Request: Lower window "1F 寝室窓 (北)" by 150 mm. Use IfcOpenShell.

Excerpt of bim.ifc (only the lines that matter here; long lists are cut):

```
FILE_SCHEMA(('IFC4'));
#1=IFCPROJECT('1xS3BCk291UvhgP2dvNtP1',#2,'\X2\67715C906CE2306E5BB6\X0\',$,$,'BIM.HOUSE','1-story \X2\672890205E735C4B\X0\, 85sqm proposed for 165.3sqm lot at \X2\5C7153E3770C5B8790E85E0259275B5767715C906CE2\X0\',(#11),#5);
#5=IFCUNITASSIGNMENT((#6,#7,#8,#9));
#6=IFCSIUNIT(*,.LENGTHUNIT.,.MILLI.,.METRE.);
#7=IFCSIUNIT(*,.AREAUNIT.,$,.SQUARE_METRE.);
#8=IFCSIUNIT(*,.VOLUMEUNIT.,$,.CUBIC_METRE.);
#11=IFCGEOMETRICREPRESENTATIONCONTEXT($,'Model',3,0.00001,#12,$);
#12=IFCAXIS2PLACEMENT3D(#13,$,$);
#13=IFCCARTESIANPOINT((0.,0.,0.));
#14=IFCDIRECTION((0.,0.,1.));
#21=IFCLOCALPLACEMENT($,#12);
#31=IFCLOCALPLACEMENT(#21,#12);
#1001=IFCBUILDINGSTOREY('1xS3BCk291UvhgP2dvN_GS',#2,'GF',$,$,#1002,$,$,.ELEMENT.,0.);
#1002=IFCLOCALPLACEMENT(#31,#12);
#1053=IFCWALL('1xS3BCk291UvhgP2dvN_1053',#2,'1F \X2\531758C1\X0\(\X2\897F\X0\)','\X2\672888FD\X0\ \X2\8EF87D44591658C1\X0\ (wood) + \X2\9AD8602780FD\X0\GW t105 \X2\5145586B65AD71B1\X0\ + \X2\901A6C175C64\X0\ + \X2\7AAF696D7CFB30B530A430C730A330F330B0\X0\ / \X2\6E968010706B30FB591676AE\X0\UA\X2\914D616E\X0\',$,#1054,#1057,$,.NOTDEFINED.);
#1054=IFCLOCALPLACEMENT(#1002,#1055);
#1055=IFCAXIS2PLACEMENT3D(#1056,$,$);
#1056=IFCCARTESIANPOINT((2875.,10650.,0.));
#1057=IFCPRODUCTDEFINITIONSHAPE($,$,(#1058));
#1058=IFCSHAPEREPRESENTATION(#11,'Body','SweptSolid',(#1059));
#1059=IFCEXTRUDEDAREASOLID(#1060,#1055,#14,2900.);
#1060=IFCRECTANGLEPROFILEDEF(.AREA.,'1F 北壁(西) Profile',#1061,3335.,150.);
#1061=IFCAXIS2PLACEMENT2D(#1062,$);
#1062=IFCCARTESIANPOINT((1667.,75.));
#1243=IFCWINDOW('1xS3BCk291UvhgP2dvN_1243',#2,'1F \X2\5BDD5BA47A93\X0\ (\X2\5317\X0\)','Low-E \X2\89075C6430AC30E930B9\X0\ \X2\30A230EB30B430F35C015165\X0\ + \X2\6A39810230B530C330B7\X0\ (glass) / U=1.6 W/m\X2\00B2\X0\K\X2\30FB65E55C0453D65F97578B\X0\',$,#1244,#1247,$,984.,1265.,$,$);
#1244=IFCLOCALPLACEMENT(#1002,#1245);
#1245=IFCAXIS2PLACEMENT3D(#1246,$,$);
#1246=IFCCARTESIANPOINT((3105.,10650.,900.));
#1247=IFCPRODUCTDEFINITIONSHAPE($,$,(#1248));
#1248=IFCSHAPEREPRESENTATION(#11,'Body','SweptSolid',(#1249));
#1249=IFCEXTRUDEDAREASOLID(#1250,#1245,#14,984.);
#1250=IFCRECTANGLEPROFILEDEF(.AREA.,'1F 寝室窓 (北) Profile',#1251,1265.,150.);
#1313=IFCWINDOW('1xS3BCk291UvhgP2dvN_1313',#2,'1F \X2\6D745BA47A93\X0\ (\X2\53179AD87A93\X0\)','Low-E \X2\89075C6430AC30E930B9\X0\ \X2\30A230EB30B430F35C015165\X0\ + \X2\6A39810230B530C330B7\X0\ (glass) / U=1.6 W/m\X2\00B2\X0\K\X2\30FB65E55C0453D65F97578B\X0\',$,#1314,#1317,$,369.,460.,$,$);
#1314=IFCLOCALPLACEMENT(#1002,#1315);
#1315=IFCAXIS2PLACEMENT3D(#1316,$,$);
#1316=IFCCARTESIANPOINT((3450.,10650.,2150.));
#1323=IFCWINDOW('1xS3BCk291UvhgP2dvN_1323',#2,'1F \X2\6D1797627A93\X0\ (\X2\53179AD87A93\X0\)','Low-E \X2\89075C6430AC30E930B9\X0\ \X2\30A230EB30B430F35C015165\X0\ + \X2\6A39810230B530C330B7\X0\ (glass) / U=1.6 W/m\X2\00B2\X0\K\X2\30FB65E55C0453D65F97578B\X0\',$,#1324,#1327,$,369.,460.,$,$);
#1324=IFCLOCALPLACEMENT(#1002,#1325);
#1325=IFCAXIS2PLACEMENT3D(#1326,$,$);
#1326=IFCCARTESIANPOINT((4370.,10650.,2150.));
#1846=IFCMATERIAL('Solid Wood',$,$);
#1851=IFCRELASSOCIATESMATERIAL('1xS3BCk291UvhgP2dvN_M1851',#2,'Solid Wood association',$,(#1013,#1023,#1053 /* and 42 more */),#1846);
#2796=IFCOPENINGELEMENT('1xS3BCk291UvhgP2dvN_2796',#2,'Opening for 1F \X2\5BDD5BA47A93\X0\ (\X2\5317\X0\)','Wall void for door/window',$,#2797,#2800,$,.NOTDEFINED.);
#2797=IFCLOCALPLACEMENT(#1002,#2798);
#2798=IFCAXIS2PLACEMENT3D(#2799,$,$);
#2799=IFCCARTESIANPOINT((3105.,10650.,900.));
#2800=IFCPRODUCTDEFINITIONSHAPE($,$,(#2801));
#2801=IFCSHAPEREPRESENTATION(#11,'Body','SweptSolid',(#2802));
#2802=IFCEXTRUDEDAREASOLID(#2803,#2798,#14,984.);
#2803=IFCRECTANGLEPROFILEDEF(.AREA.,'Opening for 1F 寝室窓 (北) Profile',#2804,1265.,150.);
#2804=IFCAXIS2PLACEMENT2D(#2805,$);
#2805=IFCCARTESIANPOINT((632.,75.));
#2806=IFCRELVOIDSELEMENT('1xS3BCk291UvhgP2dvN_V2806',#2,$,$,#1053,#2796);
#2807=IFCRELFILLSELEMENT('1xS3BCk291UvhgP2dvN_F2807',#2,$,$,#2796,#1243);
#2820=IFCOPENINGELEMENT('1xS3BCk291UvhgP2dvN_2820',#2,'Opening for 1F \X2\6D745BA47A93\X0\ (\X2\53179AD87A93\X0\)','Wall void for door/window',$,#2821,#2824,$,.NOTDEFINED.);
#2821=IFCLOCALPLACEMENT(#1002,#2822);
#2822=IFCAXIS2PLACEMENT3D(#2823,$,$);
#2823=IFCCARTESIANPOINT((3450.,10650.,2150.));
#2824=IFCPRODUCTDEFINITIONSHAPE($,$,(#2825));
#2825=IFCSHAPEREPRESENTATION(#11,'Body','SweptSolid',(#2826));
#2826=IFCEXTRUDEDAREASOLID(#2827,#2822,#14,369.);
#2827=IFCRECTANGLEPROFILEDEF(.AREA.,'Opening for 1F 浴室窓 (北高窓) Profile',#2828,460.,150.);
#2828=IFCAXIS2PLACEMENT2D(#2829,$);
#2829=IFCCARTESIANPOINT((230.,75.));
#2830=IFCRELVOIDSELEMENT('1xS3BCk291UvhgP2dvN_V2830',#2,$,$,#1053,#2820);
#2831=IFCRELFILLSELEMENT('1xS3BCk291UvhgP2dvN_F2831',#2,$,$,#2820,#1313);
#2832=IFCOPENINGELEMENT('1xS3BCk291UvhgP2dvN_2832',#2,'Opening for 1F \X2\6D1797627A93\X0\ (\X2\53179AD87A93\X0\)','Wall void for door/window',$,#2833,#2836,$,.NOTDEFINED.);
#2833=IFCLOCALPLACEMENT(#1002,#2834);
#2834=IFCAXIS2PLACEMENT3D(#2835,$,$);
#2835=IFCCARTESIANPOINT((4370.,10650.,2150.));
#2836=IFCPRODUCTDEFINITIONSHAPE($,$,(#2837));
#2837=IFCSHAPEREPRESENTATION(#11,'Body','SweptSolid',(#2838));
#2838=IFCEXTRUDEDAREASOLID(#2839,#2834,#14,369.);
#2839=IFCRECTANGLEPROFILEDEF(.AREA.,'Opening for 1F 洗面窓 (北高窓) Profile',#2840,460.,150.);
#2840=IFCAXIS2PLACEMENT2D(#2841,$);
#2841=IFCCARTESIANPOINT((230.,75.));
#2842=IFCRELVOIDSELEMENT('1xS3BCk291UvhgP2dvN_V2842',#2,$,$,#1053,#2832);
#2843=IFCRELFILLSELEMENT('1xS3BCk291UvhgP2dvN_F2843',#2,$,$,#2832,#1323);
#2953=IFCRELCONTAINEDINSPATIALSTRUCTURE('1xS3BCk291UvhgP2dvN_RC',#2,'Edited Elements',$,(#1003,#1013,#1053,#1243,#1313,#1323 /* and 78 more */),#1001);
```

```python
import numpy as np
import ifcopenshell
import ifcopenshell.api.geometry
import ifcopenshell.util.placement
import ifcopenshell.util.unit

model = ifcopenshell.open("bim.ifc")
unit_scale = ifcopenshell.util.unit.calculate_unit_scale(model)

window = model.by_guid("1xS3BCk291UvhgP2dvN_1243")
opening = window.FillsVoids[0].RelatingOpeningElement
dz = -150.0

shift = np.array([0.0, 0.0, dz])
# The window is not placed relative to its opening, so move both.
for product in (opening, window):
    matrix = ifcopenshell.util.placement.get_local_placement(product.ObjectPlacement)
    matrix[:3, 3] += shift
    ifcopenshell.api.geometry.edit_object_placement(model, product=product, matrix=matrix, is_si=False)

print(f"moved by {dz * unit_scale:+.3f} m")

model.write("bim_rev.ifc")
```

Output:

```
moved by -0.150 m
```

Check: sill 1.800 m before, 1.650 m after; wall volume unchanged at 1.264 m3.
